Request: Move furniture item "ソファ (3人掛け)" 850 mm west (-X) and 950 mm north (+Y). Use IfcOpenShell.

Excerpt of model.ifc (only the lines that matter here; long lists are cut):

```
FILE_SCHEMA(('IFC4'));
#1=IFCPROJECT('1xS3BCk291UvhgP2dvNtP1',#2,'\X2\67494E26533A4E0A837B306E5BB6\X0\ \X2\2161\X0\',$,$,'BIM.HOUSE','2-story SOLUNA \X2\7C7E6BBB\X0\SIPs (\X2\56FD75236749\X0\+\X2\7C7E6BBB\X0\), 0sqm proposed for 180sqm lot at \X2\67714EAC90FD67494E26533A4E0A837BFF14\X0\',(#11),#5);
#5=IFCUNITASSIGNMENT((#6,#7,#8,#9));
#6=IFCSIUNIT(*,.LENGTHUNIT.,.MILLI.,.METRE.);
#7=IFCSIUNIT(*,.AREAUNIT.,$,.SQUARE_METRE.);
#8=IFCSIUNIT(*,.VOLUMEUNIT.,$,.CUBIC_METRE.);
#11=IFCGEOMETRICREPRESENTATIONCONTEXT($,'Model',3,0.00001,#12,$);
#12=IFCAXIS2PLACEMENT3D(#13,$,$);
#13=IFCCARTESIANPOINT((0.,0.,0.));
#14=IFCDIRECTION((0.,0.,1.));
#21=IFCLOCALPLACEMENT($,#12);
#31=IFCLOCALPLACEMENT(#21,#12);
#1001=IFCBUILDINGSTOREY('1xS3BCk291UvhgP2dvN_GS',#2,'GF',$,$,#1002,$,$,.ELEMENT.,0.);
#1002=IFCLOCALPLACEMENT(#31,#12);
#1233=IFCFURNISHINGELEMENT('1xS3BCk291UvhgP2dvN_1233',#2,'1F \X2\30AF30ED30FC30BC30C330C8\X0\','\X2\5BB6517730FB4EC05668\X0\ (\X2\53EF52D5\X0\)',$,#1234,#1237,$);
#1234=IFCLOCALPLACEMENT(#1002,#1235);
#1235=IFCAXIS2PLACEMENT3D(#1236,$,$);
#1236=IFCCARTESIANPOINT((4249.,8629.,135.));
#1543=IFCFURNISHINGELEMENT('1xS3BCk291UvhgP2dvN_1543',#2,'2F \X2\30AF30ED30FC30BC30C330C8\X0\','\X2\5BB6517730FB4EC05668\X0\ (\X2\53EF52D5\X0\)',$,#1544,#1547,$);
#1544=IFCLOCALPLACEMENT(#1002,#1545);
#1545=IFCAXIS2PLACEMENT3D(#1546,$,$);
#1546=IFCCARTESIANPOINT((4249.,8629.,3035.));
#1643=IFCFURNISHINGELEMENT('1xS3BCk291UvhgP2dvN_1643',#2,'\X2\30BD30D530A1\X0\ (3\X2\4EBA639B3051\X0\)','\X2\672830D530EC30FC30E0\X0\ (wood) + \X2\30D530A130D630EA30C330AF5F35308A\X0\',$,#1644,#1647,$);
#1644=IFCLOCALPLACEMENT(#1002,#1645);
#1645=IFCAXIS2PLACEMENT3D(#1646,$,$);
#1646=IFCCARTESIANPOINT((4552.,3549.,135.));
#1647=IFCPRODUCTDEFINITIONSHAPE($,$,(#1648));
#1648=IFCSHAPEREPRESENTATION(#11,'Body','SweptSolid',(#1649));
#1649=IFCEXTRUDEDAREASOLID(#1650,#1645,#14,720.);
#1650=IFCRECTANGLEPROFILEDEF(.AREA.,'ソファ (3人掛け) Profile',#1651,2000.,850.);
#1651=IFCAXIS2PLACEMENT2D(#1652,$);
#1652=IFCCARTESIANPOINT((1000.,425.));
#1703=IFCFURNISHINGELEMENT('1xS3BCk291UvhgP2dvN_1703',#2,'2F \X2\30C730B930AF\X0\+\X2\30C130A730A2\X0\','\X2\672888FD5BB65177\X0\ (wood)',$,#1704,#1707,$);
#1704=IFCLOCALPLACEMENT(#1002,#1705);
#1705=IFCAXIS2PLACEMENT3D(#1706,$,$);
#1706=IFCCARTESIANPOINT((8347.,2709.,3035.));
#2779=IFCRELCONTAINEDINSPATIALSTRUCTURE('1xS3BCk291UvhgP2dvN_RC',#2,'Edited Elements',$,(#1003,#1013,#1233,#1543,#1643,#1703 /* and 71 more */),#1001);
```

```python
import ifcopenshell
import ifcopenshell.api.geometry
import ifcopenshell.util.placement
import ifcopenshell.util.unit

model = ifcopenshell.open("model.ifc")
unit_scale = ifcopenshell.util.unit.calculate_unit_scale(model)

item = model.by_guid("1xS3BCk291UvhgP2dvN_1643")
matrix = ifcopenshell.util.placement.get_local_placement(item.ObjectPlacement)
matrix[0, 3] -= 0.85 / unit_scale
matrix[1, 3] += 0.95 / unit_scale
ifcopenshell.api.geometry.edit_object_placement(model, product=item, matrix=matrix, is_si=False)

print(ifcopenshell.util.placement.get_local_placement(item.ObjectPlacement).round(3) + 0.0)

model.write("model-out.ifc")
```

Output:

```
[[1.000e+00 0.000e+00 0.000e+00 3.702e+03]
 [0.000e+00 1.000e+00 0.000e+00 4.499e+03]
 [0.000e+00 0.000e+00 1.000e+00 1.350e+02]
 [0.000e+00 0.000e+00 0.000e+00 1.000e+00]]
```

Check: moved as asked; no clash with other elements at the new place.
